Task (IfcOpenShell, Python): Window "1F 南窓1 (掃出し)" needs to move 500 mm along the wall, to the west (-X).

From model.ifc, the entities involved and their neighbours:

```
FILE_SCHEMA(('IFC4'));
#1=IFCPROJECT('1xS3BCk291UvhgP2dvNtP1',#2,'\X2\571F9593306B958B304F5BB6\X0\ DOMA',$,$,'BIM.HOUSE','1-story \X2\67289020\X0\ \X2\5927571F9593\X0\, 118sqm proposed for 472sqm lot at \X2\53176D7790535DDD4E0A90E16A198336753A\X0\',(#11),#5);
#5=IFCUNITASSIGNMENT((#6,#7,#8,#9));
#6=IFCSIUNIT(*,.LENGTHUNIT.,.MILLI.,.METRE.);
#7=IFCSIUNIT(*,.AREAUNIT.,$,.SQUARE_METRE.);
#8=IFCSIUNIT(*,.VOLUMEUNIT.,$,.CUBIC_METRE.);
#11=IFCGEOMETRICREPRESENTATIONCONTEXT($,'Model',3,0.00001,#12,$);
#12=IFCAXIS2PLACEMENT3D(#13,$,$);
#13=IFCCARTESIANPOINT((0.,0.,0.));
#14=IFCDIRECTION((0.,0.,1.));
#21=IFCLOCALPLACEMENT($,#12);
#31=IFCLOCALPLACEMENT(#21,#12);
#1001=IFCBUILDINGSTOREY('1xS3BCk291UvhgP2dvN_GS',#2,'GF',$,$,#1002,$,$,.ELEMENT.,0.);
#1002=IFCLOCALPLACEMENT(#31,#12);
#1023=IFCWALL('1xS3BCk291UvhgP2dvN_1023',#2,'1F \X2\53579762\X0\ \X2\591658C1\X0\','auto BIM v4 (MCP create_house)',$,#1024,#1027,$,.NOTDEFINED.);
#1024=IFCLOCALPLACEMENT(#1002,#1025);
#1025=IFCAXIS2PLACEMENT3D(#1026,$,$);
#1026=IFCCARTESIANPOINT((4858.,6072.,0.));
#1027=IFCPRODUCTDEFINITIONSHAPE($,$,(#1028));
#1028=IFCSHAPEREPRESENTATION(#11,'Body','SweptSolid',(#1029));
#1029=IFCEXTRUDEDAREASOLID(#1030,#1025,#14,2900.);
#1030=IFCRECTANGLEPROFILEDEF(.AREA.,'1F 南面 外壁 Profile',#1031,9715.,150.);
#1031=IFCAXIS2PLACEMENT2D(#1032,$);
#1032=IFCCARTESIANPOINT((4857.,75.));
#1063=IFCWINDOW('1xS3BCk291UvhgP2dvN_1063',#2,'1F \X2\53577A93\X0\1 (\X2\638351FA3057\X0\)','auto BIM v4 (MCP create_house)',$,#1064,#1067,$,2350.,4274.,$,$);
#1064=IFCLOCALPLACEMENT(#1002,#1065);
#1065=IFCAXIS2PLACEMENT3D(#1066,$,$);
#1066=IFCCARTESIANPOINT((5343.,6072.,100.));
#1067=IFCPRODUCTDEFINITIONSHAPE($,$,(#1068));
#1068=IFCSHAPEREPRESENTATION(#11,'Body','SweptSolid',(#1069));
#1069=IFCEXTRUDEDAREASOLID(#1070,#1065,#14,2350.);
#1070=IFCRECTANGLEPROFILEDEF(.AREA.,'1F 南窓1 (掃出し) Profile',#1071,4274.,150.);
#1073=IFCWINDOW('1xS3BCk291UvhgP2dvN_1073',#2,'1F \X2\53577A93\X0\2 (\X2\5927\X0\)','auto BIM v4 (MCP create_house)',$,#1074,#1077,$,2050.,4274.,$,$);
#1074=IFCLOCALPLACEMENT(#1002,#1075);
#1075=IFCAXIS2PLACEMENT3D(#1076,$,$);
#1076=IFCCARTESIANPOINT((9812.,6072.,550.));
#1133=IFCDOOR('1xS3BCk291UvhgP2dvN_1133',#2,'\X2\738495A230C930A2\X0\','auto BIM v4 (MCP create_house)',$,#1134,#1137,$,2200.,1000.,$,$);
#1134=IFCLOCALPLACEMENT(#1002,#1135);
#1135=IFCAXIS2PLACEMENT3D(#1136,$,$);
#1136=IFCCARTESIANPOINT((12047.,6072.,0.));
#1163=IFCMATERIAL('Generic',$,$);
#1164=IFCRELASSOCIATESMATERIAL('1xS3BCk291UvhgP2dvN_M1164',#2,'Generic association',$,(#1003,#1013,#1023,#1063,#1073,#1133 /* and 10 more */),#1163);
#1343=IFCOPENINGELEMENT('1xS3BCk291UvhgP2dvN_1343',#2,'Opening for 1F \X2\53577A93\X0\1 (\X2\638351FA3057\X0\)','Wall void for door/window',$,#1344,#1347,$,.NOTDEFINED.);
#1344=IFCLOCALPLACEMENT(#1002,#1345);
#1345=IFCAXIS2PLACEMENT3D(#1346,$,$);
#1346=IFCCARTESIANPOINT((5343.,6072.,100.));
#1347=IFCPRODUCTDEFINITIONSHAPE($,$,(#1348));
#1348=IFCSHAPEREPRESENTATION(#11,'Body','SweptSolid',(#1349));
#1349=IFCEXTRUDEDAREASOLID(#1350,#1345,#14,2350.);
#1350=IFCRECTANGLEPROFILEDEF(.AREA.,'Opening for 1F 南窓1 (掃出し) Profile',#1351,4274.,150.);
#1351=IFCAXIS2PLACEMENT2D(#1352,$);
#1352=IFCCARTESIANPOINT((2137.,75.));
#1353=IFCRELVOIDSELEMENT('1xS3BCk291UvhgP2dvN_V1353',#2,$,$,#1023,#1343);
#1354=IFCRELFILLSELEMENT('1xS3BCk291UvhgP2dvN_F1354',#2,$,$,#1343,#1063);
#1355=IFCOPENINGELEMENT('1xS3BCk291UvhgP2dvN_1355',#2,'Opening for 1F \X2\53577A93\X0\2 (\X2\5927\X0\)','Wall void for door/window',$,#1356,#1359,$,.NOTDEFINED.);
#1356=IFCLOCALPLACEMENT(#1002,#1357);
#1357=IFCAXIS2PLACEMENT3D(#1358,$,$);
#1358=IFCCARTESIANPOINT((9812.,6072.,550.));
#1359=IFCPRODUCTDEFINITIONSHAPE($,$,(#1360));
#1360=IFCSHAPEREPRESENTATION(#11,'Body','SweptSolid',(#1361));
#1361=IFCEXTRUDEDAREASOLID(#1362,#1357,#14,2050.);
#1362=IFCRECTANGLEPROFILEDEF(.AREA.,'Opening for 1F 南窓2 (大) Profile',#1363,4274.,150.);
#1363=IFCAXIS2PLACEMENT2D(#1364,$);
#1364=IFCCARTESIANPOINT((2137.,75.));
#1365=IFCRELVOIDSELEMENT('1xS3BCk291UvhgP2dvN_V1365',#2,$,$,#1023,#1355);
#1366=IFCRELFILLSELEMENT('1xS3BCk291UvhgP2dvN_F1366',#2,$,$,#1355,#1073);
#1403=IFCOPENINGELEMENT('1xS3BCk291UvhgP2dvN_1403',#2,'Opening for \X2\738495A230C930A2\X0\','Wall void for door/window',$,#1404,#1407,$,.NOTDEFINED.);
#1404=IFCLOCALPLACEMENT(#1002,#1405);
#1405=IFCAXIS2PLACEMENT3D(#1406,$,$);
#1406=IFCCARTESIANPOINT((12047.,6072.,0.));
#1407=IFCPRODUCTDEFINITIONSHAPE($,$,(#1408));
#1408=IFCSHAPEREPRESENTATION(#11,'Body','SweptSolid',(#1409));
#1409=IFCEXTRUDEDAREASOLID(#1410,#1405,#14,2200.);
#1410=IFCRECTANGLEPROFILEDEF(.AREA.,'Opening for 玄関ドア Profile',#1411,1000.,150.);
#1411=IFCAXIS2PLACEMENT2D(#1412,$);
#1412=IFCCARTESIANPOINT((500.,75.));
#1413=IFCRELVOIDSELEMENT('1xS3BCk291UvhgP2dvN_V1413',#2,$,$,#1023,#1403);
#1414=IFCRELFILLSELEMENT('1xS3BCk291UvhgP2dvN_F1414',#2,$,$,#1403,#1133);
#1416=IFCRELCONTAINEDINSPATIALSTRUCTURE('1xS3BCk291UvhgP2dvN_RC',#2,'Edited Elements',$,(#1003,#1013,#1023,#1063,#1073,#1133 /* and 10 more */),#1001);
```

```python
import ifcopenshell
import ifcopenshell.api.geometry
import ifcopenshell.util.placement
import ifcopenshell.util.unit

model = ifcopenshell.open("model.ifc")
unit_scale = ifcopenshell.util.unit.calculate_unit_scale(model)

window = model.by_guid("1xS3BCk291UvhgP2dvN_1063")
opening = window.FillsVoids[0].RelatingOpeningElement
wall = opening.VoidsElements[0].RelatingBuildingElement

wall_matrix = ifcopenshell.util.placement.get_local_placement(wall.ObjectPlacement)
shift = wall_matrix[:3, 0] * -0.5 / unit_scale
before = ifcopenshell.util.placement.get_local_placement(window.ObjectPlacement)[:3, 3].copy()

# The window is not placed relative to its opening, so move both.
for product in (opening, window):
    matrix = ifcopenshell.util.placement.get_local_placement(product.ObjectPlacement)
    matrix[:3, 3] += shift
    ifcopenshell.api.geometry.edit_object_placement(model, product=product, matrix=matrix, is_si=False)

after = ifcopenshell.util.placement.get_local_placement(window.ObjectPlacement)[:3, 3]
print("window moved by", (after - before).round(3) + 0.0)

model.write("model_updated.ifc")
```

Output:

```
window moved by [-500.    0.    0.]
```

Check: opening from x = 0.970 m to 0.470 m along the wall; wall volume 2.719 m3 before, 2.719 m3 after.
